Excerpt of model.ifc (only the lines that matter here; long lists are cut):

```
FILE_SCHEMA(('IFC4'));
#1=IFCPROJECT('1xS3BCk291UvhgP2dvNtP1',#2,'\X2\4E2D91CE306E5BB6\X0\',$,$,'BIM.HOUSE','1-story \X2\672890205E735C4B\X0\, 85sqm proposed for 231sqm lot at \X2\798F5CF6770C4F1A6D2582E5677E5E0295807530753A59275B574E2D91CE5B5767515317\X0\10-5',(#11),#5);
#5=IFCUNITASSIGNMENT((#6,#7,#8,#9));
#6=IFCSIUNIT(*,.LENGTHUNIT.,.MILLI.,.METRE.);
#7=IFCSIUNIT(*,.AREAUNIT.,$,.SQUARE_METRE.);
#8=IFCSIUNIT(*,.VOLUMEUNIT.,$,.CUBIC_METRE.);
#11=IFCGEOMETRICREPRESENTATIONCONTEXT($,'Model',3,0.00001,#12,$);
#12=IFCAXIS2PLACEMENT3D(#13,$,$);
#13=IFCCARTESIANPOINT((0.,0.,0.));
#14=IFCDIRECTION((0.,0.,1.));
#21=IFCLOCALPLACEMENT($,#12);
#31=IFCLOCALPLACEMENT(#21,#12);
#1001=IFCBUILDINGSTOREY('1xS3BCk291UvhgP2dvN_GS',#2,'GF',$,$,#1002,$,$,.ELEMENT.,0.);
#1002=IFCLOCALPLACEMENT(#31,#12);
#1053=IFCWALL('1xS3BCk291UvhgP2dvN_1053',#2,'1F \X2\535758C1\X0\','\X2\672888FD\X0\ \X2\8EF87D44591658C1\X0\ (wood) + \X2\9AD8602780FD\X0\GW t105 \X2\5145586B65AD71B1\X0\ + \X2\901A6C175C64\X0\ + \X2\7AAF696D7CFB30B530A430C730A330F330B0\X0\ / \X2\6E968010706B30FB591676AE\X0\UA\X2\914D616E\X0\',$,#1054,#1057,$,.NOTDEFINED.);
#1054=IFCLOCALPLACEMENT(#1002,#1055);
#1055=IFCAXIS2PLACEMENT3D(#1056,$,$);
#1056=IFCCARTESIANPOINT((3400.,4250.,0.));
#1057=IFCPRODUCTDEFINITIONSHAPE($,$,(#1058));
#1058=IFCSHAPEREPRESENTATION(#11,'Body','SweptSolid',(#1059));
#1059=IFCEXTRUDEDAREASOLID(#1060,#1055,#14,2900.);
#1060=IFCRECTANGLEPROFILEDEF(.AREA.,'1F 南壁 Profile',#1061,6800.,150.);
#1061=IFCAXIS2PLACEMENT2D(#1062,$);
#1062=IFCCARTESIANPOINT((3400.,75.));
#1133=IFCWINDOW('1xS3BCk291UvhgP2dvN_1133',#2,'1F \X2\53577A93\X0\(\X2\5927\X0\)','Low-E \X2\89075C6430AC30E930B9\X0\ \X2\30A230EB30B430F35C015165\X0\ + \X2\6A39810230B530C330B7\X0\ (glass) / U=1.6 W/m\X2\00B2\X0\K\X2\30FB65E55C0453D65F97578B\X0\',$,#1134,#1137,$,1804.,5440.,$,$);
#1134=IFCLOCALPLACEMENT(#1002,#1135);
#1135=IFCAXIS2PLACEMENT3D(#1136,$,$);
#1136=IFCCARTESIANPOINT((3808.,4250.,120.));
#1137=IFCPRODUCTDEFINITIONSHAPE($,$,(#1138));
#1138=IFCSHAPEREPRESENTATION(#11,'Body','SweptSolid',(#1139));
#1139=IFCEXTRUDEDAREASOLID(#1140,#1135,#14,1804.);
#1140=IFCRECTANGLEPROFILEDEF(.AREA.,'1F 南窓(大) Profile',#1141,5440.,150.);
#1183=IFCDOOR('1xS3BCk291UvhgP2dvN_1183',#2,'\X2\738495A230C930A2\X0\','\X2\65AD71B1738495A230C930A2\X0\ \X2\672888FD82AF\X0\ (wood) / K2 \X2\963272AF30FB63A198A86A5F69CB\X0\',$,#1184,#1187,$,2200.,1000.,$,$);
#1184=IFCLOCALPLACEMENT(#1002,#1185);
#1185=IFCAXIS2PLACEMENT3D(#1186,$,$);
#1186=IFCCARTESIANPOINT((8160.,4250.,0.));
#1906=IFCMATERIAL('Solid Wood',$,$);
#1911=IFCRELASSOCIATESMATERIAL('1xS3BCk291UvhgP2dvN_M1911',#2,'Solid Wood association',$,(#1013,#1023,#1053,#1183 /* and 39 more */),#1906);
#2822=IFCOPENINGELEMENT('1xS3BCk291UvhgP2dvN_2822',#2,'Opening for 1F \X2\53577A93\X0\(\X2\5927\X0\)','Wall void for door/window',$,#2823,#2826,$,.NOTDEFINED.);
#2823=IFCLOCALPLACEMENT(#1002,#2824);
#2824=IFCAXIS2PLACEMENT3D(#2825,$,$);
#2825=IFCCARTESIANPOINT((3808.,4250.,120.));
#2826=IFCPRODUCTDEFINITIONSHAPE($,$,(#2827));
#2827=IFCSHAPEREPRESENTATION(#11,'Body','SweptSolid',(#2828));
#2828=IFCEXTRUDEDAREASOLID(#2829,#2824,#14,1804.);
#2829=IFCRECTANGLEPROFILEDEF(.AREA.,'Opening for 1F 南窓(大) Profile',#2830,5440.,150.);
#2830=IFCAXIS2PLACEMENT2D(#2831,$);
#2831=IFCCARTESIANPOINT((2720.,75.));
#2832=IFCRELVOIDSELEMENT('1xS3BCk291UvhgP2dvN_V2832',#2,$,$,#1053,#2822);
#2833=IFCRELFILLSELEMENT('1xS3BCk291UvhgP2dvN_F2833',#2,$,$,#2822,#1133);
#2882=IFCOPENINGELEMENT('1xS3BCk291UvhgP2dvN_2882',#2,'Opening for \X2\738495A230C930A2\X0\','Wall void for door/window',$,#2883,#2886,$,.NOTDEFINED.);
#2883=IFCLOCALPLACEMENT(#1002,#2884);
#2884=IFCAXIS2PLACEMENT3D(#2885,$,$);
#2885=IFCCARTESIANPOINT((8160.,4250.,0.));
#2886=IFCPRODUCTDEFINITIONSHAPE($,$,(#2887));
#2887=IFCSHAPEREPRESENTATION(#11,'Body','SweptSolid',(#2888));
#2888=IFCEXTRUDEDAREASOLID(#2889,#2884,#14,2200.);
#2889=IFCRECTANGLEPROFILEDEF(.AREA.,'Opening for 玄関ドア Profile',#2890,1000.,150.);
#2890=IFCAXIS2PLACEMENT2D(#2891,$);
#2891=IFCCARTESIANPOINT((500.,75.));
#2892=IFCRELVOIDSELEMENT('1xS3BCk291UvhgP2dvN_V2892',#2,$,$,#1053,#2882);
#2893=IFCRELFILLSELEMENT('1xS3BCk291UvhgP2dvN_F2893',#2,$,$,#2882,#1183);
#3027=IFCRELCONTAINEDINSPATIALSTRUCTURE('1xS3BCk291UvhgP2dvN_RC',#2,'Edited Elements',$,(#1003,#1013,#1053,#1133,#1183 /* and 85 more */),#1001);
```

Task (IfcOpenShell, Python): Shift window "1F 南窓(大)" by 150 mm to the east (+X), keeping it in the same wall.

```python
import ifcopenshell
import ifcopenshell.api.geometry
import ifcopenshell.util.placement
import ifcopenshell.util.unit

model = ifcopenshell.open("model.ifc")
unit_scale = ifcopenshell.util.unit.calculate_unit_scale(model)

window = model.by_guid("1xS3BCk291UvhgP2dvN_1133")
opening = window.FillsVoids[0].RelatingOpeningElement
wall = opening.VoidsElements[0].RelatingBuildingElement

wall_matrix = ifcopenshell.util.placement.get_local_placement(wall.ObjectPlacement)
shift = wall_matrix[:3, 0] * 0.15 / unit_scale
before = ifcopenshell.util.placement.get_local_placement(window.ObjectPlacement)[:3, 3].copy()

# The window is not placed relative to its opening, so move both.
for product in (opening, window):
    matrix = ifcopenshell.util.placement.get_local_placement(product.ObjectPlacement)
    matrix[:3, 3] += shift
    ifcopenshell.api.geometry.edit_object_placement(model, product=product, matrix=matrix, is_si=False)

after = ifcopenshell.util.placement.get_local_placement(window.ObjectPlacement)[:3, 3]
print("window moved by", (after - before).round(3) + 0.0)

model.write("model_rev.ifc")
```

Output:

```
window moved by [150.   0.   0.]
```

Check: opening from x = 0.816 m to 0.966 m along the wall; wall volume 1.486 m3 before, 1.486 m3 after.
